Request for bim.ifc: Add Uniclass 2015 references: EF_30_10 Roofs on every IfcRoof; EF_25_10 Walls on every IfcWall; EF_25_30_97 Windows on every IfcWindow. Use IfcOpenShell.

First a look at what the model holds.

```python
import ifcopenshell

model = ifcopenshell.open("bim.ifc")
print(model.schema)
print("classifications:", [c.Name for c in model.by_type("IfcClassification")])
for ifc_class in ("IfcDoor", "IfcRoof", "IfcStair", "IfcWall", "IfcWindow"):
    print(ifc_class, len(model.by_type(ifc_class)))
```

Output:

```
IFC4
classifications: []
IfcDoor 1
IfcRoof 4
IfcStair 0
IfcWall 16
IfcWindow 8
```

```python
import ifcopenshell
import ifcopenshell.api.classification

model = ifcopenshell.open("bim.ifc")

system = ifcopenshell.api.classification.add_classification(model, classification="Uniclass 2015")

codes = {
    "IfcRoof": ("EF_30_10", "Roofs"),
    "IfcWall": ("EF_25_10", "Walls"),
    "IfcWindow": ("EF_25_30_97", "Windows"),
}
for ifc_class, (code, name) in codes.items():
    products = model.by_type(ifc_class)
    ifcopenshell.api.classification.add_reference(
        model, products=products, classification=system, identification=code, name=name
    )
    print(code, len(products))

model.write("bim_updated.ifc")
```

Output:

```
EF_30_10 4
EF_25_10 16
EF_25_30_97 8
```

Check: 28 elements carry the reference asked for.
